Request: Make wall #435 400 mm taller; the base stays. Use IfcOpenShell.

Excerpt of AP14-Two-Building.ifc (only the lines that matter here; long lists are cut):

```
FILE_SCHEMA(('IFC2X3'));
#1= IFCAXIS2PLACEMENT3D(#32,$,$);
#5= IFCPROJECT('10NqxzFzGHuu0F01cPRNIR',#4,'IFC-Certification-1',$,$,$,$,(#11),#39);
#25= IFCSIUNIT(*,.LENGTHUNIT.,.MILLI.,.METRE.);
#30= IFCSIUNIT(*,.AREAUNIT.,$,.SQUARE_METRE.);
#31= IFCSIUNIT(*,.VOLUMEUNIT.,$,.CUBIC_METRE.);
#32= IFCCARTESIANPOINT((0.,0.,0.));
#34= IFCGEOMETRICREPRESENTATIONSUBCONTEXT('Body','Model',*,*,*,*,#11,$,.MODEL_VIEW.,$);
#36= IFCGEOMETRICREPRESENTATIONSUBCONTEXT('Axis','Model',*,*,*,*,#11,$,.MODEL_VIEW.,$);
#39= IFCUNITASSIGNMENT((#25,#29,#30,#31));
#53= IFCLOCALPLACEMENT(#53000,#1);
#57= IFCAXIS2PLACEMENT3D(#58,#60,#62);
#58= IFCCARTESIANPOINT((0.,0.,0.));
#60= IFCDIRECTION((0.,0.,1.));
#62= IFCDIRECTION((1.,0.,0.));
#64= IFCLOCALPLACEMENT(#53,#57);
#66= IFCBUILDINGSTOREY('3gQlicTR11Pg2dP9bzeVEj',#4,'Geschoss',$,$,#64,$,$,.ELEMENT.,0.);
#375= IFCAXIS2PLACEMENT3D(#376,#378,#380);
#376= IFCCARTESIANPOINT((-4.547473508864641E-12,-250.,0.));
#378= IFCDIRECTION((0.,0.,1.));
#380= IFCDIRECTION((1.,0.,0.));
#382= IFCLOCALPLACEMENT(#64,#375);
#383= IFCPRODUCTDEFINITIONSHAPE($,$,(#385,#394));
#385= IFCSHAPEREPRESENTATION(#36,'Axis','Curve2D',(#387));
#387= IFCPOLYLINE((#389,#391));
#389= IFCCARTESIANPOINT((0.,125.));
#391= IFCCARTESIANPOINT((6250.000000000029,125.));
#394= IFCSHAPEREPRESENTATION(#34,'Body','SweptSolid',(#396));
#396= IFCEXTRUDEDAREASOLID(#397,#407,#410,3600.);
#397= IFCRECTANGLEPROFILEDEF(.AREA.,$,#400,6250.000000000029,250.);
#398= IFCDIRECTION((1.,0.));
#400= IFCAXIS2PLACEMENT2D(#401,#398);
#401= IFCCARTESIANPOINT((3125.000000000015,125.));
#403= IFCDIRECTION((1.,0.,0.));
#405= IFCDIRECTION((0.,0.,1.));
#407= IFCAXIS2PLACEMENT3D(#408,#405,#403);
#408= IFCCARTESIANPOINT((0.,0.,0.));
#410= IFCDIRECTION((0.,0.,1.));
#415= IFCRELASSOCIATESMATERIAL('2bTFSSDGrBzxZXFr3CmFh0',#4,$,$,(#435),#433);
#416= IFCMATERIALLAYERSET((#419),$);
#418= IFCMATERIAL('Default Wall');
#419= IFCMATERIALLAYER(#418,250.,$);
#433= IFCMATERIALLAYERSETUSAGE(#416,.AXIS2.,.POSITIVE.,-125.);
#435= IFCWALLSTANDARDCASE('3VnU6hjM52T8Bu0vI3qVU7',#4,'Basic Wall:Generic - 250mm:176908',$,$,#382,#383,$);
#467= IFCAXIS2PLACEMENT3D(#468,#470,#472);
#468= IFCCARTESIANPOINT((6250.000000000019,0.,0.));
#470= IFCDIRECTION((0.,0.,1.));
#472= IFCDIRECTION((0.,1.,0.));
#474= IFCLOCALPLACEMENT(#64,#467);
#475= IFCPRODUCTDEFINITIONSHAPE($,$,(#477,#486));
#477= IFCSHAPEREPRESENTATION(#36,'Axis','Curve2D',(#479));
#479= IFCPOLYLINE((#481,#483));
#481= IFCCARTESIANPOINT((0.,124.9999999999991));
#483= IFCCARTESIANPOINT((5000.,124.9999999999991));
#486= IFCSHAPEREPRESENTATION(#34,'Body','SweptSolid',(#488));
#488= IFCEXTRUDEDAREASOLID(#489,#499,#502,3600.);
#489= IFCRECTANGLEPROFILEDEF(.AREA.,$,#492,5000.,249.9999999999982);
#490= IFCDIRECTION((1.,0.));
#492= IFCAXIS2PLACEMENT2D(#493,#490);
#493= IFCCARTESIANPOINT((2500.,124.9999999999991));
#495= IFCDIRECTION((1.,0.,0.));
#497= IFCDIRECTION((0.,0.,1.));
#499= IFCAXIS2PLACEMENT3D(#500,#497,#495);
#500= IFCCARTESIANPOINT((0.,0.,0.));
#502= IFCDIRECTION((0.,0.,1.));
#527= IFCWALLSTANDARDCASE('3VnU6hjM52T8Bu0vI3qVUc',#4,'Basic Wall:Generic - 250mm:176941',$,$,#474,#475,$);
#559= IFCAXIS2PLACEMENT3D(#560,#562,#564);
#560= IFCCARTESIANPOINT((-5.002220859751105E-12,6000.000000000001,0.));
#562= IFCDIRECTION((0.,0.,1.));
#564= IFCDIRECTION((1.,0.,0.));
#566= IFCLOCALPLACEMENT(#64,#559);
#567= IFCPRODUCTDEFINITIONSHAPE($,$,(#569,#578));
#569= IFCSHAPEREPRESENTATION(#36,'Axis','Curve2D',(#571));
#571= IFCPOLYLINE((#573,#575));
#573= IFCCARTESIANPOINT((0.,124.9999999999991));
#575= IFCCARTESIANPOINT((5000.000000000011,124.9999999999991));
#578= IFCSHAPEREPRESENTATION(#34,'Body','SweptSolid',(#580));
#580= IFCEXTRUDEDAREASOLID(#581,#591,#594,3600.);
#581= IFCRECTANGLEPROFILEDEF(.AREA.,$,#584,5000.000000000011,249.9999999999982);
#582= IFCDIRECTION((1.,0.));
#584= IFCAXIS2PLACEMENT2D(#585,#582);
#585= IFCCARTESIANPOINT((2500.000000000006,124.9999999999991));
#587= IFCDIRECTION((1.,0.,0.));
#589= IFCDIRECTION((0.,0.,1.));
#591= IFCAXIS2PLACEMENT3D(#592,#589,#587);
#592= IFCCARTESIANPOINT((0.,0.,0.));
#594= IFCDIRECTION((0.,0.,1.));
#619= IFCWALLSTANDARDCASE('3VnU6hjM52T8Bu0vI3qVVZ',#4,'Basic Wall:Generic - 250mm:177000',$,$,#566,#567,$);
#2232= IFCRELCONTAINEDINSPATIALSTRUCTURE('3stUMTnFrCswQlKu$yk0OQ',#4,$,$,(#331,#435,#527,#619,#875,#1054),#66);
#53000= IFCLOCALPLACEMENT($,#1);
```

```python
import ifcopenshell
import ifcopenshell.geom
import ifcopenshell.util.representation
import ifcopenshell.util.shape
import ifcopenshell.util.unit

model = ifcopenshell.open("AP14-Two-Building.ifc")
unit_scale = ifcopenshell.util.unit.calculate_unit_scale(model)
settings = ifcopenshell.geom.settings()


def volume(element):
    """Net volume in cubic metres, openings subtracted."""
    shape = ifcopenshell.geom.create_shape(settings, element)
    return ifcopenshell.util.shape.get_volume(shape.geometry)


wall = model.by_guid("3VnU6hjM52T8Bu0vI3qVU7")
before = volume(wall)

body = ifcopenshell.util.representation.get_representation(wall, "Model", "Body")
solid = body.Items[0]
old_height = solid.Depth
solid.Depth += 0.4 / unit_scale
after = volume(wall)

print(f"height {old_height:g} -> {solid.Depth:g}, volume {before:.3f} -> {after:.3f} m3")

model.write("AP14-Two-Building_edited.ifc")
```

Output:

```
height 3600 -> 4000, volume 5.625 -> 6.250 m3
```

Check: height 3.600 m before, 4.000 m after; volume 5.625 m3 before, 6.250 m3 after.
